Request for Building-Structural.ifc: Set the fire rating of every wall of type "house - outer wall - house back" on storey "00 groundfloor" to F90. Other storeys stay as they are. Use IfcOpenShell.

First a look at what the model holds.

```python
import ifcopenshell
import ifcopenshell.util.element

model = ifcopenshell.open("Building-Structural.ifc")
print(model.schema)
storey = next(s for s in model.by_type("IfcBuildingStorey") if s.Name == "00 groundfloor")
walls = [e for e in ifcopenshell.util.element.get_decomposition(storey) if e.is_a("IfcWall")]
seen = {}
for e in walls:
    element_type = ifcopenshell.util.element.get_type(e)
    key = (element_type.Name if element_type != e and element_type else None, ifcopenshell.util.element.get_pset(e, "Pset_WallCommon", "FireRating"))
    seen[key] = seen.get(key, 0) + 1
for (name, value), count in sorted(seen.items(), key=str):
    print(count, "x", name, "|", value)
```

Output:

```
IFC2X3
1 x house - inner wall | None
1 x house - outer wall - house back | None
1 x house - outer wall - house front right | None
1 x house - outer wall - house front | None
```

```python
import ifcopenshell
import ifcopenshell.api.pset
import ifcopenshell.util.element

model = ifcopenshell.open("Building-Structural.ifc")

storey = next(s for s in model.by_type("IfcBuildingStorey") if s.Name == "00 groundfloor")
walls = [e for e in ifcopenshell.util.element.get_decomposition(storey) if e.is_a("IfcWall")]

count = 0
for e in walls:
    element_type = ifcopenshell.util.element.get_type(e)
    if element_type in (None, e) or element_type.Name != "house - outer wall - house back":
        continue
    # add_pset returns the element's existing set when there is one.
    pset = ifcopenshell.api.pset.add_pset(model, product=e, name="Pset_WallCommon")
    ifcopenshell.api.pset.edit_pset(model, pset=pset, properties={"FireRating": "F90"})
    count += 1

print(count, "walls updated")

model.write("Building-Structural-out.ifc")
```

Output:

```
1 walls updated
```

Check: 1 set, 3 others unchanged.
